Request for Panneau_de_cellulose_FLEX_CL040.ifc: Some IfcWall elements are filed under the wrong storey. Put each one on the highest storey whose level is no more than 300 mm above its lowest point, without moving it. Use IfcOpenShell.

First a look at what the model holds.

```python
import ifcopenshell
import ifcopenshell.util.element
import ifcopenshell.util.placement

model = ifcopenshell.open("Panneau_de_cellulose_FLEX_CL040.ifc")
print(model.schema)
for storey in model.by_type("IfcBuildingStorey"):
    level = ifcopenshell.util.placement.get_storey_elevation(storey)
    count = sum(e.is_a("IfcWall") for e in ifcopenshell.util.element.get_contained(storey))
    print(storey.id(), storey.Name, round(level, 3), count, sep=" | ")
```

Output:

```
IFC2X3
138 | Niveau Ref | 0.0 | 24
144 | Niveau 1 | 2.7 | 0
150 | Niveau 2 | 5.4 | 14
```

```python
import ifcopenshell
import ifcopenshell.api.spatial
import ifcopenshell.geom
import ifcopenshell.util.element
import ifcopenshell.util.placement
import ifcopenshell.util.shape
import ifcopenshell.util.unit

model = ifcopenshell.open("Panneau_de_cellulose_FLEX_CL040.ifc")
unit_scale = ifcopenshell.util.unit.calculate_unit_scale(model)
settings = ifcopenshell.geom.settings()

levels = sorted(
    ((ifcopenshell.util.placement.get_storey_elevation(s) * unit_scale, s) for s in model.by_type("IfcBuildingStorey")),
    key=lambda pair: pair[0],
)

for e in model.by_type("IfcWall"):
    current = e.ContainedInStructure[0].RelatingStructure if e.ContainedInStructure else None
    if current is None or not current.is_a("IfcBuildingStorey"):
        continue
    shape = ifcopenshell.geom.create_shape(settings, e)
    bottom = ifcopenshell.util.shape.get_shape_bottom_elevation(shape, shape.geometry)
    below = [s for level, s in levels if level <= bottom + 0.3]
    storey = below[-1] if below else levels[0][1]
    if storey != current:
        # assign_container keeps the world position.
        ifcopenshell.api.spatial.assign_container(model, products=[e], relating_structure=storey)
        print(e.id(), current.Name, "->", storey.Name)

model.write("Panneau_de_cellulose_FLEX_CL040-out.ifc")
```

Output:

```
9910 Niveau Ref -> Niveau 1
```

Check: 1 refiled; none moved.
